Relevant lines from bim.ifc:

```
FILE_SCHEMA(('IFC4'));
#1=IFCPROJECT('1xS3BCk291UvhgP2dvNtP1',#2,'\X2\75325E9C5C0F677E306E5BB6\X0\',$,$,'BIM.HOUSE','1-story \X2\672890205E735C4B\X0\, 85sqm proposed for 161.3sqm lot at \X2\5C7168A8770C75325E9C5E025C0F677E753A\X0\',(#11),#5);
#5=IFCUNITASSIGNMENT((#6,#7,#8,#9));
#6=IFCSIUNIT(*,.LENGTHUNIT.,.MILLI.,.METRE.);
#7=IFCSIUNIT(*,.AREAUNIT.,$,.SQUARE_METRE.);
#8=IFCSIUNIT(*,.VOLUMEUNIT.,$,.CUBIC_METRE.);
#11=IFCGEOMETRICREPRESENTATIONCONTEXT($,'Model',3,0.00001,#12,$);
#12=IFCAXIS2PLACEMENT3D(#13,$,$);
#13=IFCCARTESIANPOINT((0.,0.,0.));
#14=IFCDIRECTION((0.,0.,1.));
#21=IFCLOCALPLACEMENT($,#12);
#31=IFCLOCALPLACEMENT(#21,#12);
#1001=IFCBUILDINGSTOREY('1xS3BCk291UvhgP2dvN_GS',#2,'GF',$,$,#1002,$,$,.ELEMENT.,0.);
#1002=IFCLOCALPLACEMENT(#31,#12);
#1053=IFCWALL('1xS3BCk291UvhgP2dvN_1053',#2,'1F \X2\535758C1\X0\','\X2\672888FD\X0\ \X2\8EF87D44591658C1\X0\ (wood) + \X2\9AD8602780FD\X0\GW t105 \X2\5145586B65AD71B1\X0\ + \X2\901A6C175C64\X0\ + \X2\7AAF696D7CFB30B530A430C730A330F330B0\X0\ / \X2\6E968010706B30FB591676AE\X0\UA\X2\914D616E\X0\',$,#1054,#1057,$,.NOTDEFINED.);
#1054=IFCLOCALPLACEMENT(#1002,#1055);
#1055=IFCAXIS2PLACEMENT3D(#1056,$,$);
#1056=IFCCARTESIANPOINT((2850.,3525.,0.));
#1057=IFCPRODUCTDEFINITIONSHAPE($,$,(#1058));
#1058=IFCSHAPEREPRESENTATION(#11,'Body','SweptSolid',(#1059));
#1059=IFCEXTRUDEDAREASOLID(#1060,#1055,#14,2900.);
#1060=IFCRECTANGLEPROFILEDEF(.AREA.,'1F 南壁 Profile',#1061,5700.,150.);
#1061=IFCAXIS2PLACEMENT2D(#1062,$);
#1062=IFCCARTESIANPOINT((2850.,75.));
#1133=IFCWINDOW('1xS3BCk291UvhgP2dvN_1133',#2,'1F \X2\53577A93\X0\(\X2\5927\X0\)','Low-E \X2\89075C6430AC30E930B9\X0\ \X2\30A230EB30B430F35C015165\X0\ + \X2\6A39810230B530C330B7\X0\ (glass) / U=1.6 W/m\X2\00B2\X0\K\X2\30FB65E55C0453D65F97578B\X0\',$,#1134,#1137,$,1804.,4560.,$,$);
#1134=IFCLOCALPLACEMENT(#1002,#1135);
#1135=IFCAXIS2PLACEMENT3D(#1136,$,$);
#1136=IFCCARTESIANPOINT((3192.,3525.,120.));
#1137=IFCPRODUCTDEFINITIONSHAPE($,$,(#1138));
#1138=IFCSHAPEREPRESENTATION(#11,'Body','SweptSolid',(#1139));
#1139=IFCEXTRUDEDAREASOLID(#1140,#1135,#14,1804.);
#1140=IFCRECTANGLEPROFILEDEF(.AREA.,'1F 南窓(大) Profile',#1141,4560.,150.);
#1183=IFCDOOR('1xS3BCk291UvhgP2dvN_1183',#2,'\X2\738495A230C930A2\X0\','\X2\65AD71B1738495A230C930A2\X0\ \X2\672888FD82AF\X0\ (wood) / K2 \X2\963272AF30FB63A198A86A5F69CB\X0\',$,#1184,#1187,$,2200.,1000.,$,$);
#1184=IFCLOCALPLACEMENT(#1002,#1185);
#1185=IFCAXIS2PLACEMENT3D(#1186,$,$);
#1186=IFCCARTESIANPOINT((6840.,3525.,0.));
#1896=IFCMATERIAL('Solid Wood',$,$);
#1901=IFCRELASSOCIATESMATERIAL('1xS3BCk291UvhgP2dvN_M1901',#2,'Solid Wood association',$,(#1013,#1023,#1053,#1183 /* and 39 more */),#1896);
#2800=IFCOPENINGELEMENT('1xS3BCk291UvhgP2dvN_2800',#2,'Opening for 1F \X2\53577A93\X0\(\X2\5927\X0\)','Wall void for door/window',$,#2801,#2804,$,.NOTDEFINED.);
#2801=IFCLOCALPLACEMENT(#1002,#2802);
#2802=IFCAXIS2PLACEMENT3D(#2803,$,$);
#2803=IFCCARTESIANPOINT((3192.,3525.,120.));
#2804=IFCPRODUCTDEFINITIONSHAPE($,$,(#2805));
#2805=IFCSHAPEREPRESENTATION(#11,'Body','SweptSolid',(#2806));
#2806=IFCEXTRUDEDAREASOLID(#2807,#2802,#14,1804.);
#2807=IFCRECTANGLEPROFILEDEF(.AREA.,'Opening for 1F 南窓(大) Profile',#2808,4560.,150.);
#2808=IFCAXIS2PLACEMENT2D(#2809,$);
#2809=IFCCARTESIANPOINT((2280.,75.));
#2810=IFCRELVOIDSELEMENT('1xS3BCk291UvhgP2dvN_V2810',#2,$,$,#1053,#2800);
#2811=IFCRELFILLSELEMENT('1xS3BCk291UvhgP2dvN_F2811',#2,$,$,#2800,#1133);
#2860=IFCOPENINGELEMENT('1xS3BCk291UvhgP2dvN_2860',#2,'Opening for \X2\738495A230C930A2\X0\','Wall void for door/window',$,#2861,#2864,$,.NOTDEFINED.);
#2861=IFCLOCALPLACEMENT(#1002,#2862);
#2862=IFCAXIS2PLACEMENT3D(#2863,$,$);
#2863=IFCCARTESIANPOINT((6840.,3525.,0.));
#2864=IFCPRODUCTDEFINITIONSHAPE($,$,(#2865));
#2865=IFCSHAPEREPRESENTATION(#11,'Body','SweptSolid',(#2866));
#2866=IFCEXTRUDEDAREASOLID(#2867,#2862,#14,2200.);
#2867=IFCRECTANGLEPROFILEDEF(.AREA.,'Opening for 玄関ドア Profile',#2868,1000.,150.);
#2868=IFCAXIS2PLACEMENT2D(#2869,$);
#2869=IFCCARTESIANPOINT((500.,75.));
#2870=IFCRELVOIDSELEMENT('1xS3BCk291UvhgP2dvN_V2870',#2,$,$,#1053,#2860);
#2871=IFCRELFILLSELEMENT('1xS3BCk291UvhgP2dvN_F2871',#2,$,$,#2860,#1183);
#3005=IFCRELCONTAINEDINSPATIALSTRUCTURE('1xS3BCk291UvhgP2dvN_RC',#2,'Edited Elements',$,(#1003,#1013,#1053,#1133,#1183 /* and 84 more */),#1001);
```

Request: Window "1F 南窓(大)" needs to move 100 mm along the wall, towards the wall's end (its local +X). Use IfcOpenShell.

```python
import ifcopenshell
import ifcopenshell.api.geometry
import ifcopenshell.util.placement

model = ifcopenshell.open("bim.ifc")

window = model.by_guid("1xS3BCk291UvhgP2dvN_1133")
opening = window.FillsVoids[0].RelatingOpeningElement
wall = opening.VoidsElements[0].RelatingBuildingElement

wall_matrix = ifcopenshell.util.placement.get_local_placement(wall.ObjectPlacement)
shift = wall_matrix[:3, 0] * 100.0
before = ifcopenshell.util.placement.get_local_placement(window.ObjectPlacement)[:3, 3].copy()

# The window is not placed relative to its opening, so move both.
for product in (opening, window):
    matrix = ifcopenshell.util.placement.get_local_placement(product.ObjectPlacement)
    matrix[:3, 3] += shift
    ifcopenshell.api.geometry.edit_object_placement(model, product=product, matrix=matrix, is_si=False)

after = ifcopenshell.util.placement.get_local_placement(window.ObjectPlacement)[:3, 3]
print("window moved by", (after - before).round(3) + 0.0)

model.write("bim_updated.ifc")
```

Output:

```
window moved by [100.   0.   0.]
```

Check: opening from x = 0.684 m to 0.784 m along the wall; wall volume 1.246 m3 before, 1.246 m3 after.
